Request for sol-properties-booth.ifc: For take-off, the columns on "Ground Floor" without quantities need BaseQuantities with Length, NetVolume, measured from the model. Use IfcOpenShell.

First a look at what the model holds.

```python
import ifcopenshell
import ifcopenshell.util.element
import ifcopenshell.util.unit

model = ifcopenshell.open("sol-properties-booth.ifc")
print(model.schema)
for unit_type in ("LENGTHUNIT", "AREAUNIT", "VOLUMEUNIT"):
    print(unit_type, ifcopenshell.util.unit.calculate_unit_scale(model, unit_type))
storey = next(s for s in model.by_type("IfcBuildingStorey") if s.Name == "Ground Floor")
columns = [e for e in ifcopenshell.util.element.get_decomposition(storey) if e.is_a("IfcColumn")]
for e in sorted(columns, key=lambda e: e.id()):
    print(e.id(), e.is_a(), e.Name, list(ifcopenshell.util.element.get_psets(e, qtos_only=True)), sep=" | ")
```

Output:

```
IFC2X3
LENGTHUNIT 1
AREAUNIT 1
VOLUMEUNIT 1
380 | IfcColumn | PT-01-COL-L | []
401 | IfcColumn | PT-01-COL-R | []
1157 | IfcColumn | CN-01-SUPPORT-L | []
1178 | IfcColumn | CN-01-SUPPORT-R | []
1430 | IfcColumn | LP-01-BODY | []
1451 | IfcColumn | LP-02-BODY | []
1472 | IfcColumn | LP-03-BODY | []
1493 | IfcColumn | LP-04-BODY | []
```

```python
import ifcopenshell
import ifcopenshell.api.pset
import ifcopenshell.geom
import ifcopenshell.util.element
import ifcopenshell.util.shape
import ifcopenshell.util.unit

model = ifcopenshell.open("sol-properties-booth.ifc")
unit_scale = ifcopenshell.util.unit.calculate_unit_scale(model)
volume_scale = ifcopenshell.util.unit.calculate_unit_scale(model, "VOLUMEUNIT")
settings = ifcopenshell.geom.settings()

storey = next(s for s in model.by_type("IfcBuildingStorey") if s.Name == "Ground Floor")
columns = [e for e in ifcopenshell.util.element.get_decomposition(storey) if e.is_a("IfcColumn")]

for e in sorted(columns, key=lambda e: e.id()):
    if ifcopenshell.util.element.get_psets(e, qtos_only=True, should_inherit=False):
        continue
    # Geometry comes back in metres, in the element's own axes.
    shape = ifcopenshell.geom.create_shape(settings, e)
    values = {
        "Length": ifcopenshell.util.shape.get_z(shape.geometry) / unit_scale,
        "NetVolume": ifcopenshell.util.shape.get_volume(shape.geometry) / volume_scale,
    }
    qto = ifcopenshell.api.pset.add_qto(model, product=e, name="BaseQuantities")
    ifcopenshell.api.pset.edit_qto(model, qto=qto, properties=values)
    print(e.id(), {k: round(v, 3) for k, v in values.items()})

model.write("sol-properties-booth_rev.ifc")
```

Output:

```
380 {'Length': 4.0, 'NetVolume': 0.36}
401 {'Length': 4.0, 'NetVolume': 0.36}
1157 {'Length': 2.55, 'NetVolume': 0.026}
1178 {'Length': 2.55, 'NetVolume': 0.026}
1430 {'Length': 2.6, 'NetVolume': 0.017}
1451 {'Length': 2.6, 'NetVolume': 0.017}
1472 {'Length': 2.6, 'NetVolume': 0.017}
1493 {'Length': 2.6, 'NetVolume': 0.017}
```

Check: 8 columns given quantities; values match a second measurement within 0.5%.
